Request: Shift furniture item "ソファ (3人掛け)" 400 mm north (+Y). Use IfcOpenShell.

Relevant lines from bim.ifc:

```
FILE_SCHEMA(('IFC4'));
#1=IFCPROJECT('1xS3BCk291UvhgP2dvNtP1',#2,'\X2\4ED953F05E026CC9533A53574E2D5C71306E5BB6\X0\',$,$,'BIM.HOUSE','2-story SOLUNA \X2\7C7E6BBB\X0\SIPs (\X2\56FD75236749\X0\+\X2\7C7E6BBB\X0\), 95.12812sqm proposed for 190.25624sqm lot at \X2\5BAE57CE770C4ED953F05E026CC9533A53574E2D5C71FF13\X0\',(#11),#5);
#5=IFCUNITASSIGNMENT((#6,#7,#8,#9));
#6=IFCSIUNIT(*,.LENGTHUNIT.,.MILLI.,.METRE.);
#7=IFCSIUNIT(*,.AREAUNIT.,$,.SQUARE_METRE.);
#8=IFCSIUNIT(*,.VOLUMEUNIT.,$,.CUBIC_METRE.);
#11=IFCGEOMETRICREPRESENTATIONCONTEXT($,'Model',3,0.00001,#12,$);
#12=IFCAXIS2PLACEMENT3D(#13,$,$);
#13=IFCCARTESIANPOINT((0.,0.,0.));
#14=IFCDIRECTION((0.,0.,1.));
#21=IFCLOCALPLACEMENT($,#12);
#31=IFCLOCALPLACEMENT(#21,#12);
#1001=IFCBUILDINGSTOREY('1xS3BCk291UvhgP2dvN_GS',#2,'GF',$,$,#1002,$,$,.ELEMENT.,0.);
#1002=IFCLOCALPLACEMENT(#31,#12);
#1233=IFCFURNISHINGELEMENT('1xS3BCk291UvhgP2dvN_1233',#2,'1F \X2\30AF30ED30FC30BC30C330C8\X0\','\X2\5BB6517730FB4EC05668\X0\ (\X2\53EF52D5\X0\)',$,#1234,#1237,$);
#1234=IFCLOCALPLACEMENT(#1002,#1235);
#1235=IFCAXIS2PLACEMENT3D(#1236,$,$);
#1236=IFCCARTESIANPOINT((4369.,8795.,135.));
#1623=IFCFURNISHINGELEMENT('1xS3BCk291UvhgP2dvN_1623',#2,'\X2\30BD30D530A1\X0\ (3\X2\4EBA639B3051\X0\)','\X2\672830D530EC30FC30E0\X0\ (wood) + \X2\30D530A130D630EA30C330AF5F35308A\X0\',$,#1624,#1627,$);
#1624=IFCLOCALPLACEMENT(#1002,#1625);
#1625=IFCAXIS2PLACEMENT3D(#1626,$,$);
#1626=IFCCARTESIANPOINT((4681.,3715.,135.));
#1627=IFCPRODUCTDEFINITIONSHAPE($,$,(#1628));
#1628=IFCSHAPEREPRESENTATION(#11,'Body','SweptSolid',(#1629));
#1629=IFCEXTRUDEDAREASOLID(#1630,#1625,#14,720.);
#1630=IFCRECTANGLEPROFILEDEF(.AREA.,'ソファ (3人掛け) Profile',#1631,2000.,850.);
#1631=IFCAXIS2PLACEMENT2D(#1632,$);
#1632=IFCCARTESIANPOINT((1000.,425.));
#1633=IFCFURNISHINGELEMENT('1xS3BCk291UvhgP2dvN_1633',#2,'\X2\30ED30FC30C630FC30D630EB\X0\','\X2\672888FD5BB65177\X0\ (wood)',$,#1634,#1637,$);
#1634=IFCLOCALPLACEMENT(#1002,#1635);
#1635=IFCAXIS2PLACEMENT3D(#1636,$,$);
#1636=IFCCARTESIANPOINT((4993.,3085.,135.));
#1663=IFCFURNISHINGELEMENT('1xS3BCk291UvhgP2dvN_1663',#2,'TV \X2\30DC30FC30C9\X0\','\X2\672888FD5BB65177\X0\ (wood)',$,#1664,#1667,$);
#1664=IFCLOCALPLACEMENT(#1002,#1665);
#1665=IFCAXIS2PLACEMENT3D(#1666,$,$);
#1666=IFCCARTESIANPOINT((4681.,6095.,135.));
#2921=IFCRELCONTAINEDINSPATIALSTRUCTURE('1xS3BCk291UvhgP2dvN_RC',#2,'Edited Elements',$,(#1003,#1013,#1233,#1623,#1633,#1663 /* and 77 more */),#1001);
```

```python
import ifcopenshell
import ifcopenshell.api.geometry
import ifcopenshell.util.placement
import ifcopenshell.util.unit

model = ifcopenshell.open("bim.ifc")
unit_scale = ifcopenshell.util.unit.calculate_unit_scale(model)

item = model.by_guid("1xS3BCk291UvhgP2dvN_1623")
matrix = ifcopenshell.util.placement.get_local_placement(item.ObjectPlacement)
matrix[1, 3] += 0.4 / unit_scale
ifcopenshell.api.geometry.edit_object_placement(model, product=item, matrix=matrix, is_si=False)

print(ifcopenshell.util.placement.get_local_placement(item.ObjectPlacement).round(3) + 0.0)

model.write("bim_v2.ifc")
```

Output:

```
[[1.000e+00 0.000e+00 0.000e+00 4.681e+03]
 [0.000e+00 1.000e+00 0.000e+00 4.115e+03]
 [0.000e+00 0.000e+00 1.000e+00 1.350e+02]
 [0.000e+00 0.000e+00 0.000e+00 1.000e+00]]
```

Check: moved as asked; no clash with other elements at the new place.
